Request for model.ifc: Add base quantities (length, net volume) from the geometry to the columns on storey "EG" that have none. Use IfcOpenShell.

First a look at what the model holds.

```python
import ifcopenshell
import ifcopenshell.util.element
import ifcopenshell.util.unit

model = ifcopenshell.open("model.ifc")
print(model.schema)
for unit_type in ("LENGTHUNIT", "AREAUNIT", "VOLUMEUNIT"):
    print(unit_type, ifcopenshell.util.unit.calculate_unit_scale(model, unit_type))
storey = next(s for s in model.by_type("IfcBuildingStorey") if s.Name == "EG")
columns = [e for e in ifcopenshell.util.element.get_decomposition(storey) if e.is_a("IfcColumn")]
for e in sorted(columns, key=lambda e: e.id()):
    print(e.id(), e.is_a(), e.Name, list(ifcopenshell.util.element.get_psets(e, qtos_only=True)), sep=" | ")
```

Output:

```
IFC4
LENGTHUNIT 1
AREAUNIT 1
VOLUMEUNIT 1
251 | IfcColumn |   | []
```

```python
import ifcopenshell
import ifcopenshell.api.pset
import ifcopenshell.geom
import ifcopenshell.util.element
import ifcopenshell.util.shape
import ifcopenshell.util.unit

model = ifcopenshell.open("model.ifc")
unit_scale = ifcopenshell.util.unit.calculate_unit_scale(model)
volume_scale = ifcopenshell.util.unit.calculate_unit_scale(model, "VOLUMEUNIT")
settings = ifcopenshell.geom.settings()

storey = next(s for s in model.by_type("IfcBuildingStorey") if s.Name == "EG")
columns = [e for e in ifcopenshell.util.element.get_decomposition(storey) if e.is_a("IfcColumn")]

for e in sorted(columns, key=lambda e: e.id()):
    if ifcopenshell.util.element.get_psets(e, qtos_only=True, should_inherit=False):
        continue
    # Geometry comes back in metres, in the element's own axes.
    shape = ifcopenshell.geom.create_shape(settings, e)
    values = {
        "Length": ifcopenshell.util.shape.get_z(shape.geometry) / unit_scale,
        "NetVolume": ifcopenshell.util.shape.get_volume(shape.geometry) / volume_scale,
    }
    qto = ifcopenshell.api.pset.add_qto(model, product=e, name="Qto_ColumnBaseQuantities")
    ifcopenshell.api.pset.edit_qto(model, qto=qto, properties=values)
    print(e.id(), {k: round(v, 3) for k, v in values.items()})

model.write("model_updated.ifc")
```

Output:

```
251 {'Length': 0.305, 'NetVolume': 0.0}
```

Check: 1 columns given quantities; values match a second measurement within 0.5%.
